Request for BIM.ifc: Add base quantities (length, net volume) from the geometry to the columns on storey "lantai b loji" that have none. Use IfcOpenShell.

First a look at what the model holds.

```python
import ifcopenshell
import ifcopenshell.util.element
import ifcopenshell.util.unit

model = ifcopenshell.open("BIM.ifc")
print(model.schema)
for unit_type in ("LENGTHUNIT", "AREAUNIT", "VOLUMEUNIT"):
    print(unit_type, ifcopenshell.util.unit.calculate_unit_scale(model, unit_type))
storey = next(s for s in model.by_type("IfcBuildingStorey") if s.Name == "lantai b loji")
columns = [e for e in ifcopenshell.util.element.get_decomposition(storey) if e.is_a("IfcColumn")]
for e in sorted(columns, key=lambda e: e.id()):
    print(e.id(), e.is_a(), e.Name, list(ifcopenshell.util.element.get_psets(e, qtos_only=True)), sep=" | ")
```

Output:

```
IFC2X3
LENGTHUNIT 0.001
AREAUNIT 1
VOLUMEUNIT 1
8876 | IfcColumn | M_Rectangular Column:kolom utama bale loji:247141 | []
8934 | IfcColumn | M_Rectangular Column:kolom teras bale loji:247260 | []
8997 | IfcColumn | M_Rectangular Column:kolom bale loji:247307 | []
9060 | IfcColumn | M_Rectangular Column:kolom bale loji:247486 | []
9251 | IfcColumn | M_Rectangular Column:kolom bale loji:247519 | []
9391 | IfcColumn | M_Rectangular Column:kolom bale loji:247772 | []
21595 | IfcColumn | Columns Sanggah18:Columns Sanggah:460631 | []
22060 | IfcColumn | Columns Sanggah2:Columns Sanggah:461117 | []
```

```python
import ifcopenshell
import ifcopenshell.api.pset
import ifcopenshell.geom
import ifcopenshell.util.element
import ifcopenshell.util.shape
import ifcopenshell.util.unit

model = ifcopenshell.open("BIM.ifc")
unit_scale = ifcopenshell.util.unit.calculate_unit_scale(model)
volume_scale = ifcopenshell.util.unit.calculate_unit_scale(model, "VOLUMEUNIT")
settings = ifcopenshell.geom.settings()

storey = next(s for s in model.by_type("IfcBuildingStorey") if s.Name == "lantai b loji")
columns = [e for e in ifcopenshell.util.element.get_decomposition(storey) if e.is_a("IfcColumn")]

for e in sorted(columns, key=lambda e: e.id()):
    if ifcopenshell.util.element.get_psets(e, qtos_only=True, should_inherit=False):
        continue
    # Geometry comes back in metres, in the element's own axes.
    shape = ifcopenshell.geom.create_shape(settings, e)
    values = {
        "Length": ifcopenshell.util.shape.get_z(shape.geometry) / unit_scale,
        "NetVolume": ifcopenshell.util.shape.get_volume(shape.geometry) / volume_scale,
    }
    qto = ifcopenshell.api.pset.add_qto(model, product=e, name="BaseQuantities")
    ifcopenshell.api.pset.edit_qto(model, qto=qto, properties=values)
    print(e.id(), {k: round(v, 3) for k, v in values.items()})

model.write("BIM_updated.ifc")
```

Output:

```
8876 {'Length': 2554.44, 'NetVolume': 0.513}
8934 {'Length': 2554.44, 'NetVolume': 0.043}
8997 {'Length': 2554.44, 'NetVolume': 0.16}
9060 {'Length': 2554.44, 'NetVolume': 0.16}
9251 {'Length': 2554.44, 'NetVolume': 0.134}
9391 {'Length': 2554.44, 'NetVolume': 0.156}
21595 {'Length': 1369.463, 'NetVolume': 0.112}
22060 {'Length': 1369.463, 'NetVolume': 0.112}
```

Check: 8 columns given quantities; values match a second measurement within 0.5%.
